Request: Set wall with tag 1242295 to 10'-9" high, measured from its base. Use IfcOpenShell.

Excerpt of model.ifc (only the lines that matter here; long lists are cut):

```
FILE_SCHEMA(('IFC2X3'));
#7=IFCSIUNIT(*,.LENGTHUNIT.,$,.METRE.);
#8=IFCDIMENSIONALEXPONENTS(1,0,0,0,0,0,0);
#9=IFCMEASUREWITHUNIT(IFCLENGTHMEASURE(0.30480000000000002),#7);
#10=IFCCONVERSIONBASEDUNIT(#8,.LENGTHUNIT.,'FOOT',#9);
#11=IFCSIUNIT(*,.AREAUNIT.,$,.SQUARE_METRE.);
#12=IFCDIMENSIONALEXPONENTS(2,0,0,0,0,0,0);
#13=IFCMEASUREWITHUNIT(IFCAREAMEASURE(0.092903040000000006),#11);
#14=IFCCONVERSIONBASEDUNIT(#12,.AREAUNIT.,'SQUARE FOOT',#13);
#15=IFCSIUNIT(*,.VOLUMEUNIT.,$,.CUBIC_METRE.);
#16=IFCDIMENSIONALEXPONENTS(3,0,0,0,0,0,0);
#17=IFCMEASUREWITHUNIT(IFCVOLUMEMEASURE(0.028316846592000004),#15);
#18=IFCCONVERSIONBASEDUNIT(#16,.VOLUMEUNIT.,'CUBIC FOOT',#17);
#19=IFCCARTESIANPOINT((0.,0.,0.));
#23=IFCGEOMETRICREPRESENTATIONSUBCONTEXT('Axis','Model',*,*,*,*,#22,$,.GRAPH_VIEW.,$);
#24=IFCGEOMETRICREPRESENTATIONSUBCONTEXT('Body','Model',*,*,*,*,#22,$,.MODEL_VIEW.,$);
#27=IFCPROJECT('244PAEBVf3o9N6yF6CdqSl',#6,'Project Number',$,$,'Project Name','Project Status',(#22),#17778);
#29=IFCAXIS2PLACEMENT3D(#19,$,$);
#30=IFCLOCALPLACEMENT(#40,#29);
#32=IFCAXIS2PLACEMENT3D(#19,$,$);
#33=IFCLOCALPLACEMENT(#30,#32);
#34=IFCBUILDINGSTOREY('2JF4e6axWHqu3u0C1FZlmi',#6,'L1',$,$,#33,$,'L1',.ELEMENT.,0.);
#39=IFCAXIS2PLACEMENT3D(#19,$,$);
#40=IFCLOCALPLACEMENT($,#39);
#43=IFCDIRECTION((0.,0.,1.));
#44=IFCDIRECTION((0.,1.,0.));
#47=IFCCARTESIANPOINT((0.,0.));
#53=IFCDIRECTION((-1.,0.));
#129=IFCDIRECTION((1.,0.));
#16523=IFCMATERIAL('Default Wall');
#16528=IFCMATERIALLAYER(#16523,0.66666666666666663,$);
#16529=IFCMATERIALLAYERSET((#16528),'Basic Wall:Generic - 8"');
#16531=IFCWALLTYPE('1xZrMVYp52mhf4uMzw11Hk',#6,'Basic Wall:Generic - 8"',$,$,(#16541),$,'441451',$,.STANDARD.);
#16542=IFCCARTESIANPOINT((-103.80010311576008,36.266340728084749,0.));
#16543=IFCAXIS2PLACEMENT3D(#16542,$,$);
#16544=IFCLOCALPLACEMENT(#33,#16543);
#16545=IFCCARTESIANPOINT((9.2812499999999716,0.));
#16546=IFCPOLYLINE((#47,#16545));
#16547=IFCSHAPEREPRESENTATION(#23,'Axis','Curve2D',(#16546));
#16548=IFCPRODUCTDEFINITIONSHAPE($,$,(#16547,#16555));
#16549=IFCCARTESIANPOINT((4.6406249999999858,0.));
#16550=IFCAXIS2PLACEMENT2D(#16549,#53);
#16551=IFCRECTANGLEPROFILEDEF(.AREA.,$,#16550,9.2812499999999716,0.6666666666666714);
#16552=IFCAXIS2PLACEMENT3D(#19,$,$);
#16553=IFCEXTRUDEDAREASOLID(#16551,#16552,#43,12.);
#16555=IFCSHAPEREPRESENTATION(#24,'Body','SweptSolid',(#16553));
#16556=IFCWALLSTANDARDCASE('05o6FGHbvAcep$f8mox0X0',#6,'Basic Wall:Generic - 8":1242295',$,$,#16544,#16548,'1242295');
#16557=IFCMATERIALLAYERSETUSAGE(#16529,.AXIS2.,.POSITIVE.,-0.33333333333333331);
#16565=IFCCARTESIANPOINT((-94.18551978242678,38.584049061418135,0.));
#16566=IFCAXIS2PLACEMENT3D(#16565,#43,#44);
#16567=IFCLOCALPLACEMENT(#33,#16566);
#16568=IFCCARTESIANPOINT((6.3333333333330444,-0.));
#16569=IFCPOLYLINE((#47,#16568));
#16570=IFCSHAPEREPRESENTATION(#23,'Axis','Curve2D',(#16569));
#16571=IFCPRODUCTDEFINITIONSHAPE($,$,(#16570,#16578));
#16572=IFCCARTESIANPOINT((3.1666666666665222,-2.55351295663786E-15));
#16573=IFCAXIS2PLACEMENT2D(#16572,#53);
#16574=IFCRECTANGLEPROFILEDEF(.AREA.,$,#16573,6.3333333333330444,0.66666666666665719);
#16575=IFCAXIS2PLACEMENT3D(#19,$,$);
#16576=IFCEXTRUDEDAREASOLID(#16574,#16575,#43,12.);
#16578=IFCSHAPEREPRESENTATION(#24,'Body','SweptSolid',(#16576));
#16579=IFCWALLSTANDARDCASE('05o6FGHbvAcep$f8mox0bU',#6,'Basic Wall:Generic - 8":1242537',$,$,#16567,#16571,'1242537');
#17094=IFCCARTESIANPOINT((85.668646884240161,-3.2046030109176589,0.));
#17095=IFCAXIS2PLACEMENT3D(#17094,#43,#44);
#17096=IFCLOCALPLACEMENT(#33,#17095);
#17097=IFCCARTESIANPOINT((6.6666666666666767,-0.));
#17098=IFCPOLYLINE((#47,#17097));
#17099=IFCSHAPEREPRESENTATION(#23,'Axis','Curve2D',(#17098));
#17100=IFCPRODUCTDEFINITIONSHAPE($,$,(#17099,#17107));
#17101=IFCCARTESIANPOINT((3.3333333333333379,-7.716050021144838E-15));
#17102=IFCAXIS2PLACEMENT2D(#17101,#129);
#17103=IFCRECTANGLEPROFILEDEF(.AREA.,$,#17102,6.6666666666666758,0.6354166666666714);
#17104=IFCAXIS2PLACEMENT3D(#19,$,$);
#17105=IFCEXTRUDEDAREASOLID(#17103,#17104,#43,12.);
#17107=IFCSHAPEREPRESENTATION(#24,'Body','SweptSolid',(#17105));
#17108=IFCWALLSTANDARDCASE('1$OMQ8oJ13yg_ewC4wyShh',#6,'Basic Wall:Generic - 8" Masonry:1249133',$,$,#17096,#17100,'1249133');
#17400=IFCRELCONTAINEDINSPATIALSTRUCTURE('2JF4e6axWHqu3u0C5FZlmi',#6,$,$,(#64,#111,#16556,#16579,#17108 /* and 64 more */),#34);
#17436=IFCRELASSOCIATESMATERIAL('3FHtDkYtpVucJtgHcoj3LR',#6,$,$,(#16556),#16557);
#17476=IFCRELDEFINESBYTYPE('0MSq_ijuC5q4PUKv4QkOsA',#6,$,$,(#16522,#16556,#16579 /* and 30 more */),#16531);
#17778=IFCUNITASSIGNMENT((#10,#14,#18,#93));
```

```python
import ifcopenshell
import ifcopenshell.geom
import ifcopenshell.util.representation
import ifcopenshell.util.shape
import ifcopenshell.util.unit

model = ifcopenshell.open("model.ifc")
unit_scale = ifcopenshell.util.unit.calculate_unit_scale(model)
settings = ifcopenshell.geom.settings()


def volume(element):
    """Net volume in cubic metres, openings subtracted."""
    shape = ifcopenshell.geom.create_shape(settings, element)
    return ifcopenshell.util.shape.get_volume(shape.geometry)


wall = model.by_guid("05o6FGHbvAcep$f8mox0X0")
before = volume(wall)

body = ifcopenshell.util.representation.get_representation(wall, "Model", "Body")
solid = body.Items[0]
old_height = solid.Depth
solid.Depth = 129 * 0.0254 / unit_scale
after = volume(wall)

print(f"height {old_height:g} -> {solid.Depth:g}, volume {before:.3f} -> {after:.3f} m3")

model.write("model_v2.ifc")
```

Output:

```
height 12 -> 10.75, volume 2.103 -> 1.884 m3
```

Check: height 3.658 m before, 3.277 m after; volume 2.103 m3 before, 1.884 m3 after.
